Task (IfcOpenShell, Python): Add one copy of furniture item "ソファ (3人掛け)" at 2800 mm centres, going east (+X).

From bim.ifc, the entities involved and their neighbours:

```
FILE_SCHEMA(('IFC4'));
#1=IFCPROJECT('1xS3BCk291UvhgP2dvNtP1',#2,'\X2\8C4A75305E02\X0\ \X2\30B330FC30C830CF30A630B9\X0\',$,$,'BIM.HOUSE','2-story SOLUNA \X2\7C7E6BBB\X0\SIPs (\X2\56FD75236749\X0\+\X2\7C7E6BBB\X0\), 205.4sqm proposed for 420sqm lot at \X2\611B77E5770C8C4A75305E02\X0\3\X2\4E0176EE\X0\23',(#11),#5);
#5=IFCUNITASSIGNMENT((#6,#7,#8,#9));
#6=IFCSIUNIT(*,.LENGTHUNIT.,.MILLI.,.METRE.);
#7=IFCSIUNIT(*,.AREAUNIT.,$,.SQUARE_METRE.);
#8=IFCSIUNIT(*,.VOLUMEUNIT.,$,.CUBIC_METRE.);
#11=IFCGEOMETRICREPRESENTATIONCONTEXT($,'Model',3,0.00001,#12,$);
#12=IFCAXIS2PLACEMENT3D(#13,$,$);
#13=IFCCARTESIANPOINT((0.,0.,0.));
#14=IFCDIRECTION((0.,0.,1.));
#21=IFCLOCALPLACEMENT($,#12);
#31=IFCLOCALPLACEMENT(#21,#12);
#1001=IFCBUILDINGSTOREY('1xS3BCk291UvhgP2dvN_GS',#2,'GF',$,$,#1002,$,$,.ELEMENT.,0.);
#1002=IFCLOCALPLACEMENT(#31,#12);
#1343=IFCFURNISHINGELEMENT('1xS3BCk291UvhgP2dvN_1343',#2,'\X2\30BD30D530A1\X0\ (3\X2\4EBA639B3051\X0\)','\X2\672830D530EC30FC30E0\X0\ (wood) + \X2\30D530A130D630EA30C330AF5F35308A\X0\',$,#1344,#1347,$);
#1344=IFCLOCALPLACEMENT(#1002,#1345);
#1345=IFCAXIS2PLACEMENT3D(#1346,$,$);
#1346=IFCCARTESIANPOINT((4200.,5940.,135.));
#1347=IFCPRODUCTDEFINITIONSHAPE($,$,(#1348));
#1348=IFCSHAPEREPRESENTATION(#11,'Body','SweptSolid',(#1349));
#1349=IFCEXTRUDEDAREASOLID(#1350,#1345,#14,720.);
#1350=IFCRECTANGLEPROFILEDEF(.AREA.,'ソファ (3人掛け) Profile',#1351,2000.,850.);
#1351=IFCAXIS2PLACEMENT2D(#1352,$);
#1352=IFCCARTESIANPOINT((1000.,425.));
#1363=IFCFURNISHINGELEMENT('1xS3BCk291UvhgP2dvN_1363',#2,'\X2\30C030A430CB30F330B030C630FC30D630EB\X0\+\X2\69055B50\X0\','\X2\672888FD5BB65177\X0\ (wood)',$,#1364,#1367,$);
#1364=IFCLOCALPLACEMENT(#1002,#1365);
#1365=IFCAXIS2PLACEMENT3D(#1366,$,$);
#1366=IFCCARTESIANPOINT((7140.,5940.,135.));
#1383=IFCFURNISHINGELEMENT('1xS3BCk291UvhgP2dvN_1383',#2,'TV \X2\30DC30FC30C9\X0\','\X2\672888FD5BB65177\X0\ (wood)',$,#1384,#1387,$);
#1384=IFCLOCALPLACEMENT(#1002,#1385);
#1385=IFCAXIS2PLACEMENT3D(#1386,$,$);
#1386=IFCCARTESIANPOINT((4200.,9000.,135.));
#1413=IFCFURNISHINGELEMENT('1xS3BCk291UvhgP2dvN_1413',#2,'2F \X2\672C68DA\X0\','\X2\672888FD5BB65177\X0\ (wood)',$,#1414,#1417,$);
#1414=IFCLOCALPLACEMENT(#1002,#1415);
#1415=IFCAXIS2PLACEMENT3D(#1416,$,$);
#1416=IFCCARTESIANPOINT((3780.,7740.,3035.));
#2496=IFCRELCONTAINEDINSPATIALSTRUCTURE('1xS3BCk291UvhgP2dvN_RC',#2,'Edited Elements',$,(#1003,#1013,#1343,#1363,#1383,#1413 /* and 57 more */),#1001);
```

```python
import numpy as np
import ifcopenshell
import ifcopenshell.api.geometry
import ifcopenshell.api.root
import ifcopenshell.util.element
import ifcopenshell.util.placement
import ifcopenshell.util.unit

model = ifcopenshell.open("bim.ifc")
unit_scale = ifcopenshell.util.unit.calculate_unit_scale(model)


def reuse_history(source, copy):
    """copy_class also copies each property set's owner history, people and application; keep the originals."""
    for rel in copy.IsDefinedBy:
        if rel.is_a("IfcRelDefinesByProperties") and (history := rel.RelatingPropertyDefinition.OwnerHistory):
            rel.RelatingPropertyDefinition.OwnerHistory = source.OwnerHistory
            ifcopenshell.util.element.remove_deep2(model, history)


source = model.by_guid("1xS3BCk291UvhgP2dvN_1343")
base = ifcopenshell.util.placement.get_local_placement(source.ObjectPlacement)
step = np.array([1.0, 0.0, 0.0]) * 2.8 / unit_scale

for i in range(1, 2):
    copy = ifcopenshell.api.root.copy_class(model, product=source)
    copy.Representation = ifcopenshell.util.element.copy_deep(
        model, source.Representation, exclude=["IfcGeometricRepresentationContext", "IfcRepresentationMap"]
    )
    reuse_history(source, copy)
    matrix = base.copy()
    matrix[:3, 3] += i * step
    print("added at", matrix[:3, 3].round(3) + 0.0)
    ifcopenshell.api.geometry.edit_object_placement(model, product=copy, matrix=matrix, is_si=False)

model.write("bim_edited.ifc")
```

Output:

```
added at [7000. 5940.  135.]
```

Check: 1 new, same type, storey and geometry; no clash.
